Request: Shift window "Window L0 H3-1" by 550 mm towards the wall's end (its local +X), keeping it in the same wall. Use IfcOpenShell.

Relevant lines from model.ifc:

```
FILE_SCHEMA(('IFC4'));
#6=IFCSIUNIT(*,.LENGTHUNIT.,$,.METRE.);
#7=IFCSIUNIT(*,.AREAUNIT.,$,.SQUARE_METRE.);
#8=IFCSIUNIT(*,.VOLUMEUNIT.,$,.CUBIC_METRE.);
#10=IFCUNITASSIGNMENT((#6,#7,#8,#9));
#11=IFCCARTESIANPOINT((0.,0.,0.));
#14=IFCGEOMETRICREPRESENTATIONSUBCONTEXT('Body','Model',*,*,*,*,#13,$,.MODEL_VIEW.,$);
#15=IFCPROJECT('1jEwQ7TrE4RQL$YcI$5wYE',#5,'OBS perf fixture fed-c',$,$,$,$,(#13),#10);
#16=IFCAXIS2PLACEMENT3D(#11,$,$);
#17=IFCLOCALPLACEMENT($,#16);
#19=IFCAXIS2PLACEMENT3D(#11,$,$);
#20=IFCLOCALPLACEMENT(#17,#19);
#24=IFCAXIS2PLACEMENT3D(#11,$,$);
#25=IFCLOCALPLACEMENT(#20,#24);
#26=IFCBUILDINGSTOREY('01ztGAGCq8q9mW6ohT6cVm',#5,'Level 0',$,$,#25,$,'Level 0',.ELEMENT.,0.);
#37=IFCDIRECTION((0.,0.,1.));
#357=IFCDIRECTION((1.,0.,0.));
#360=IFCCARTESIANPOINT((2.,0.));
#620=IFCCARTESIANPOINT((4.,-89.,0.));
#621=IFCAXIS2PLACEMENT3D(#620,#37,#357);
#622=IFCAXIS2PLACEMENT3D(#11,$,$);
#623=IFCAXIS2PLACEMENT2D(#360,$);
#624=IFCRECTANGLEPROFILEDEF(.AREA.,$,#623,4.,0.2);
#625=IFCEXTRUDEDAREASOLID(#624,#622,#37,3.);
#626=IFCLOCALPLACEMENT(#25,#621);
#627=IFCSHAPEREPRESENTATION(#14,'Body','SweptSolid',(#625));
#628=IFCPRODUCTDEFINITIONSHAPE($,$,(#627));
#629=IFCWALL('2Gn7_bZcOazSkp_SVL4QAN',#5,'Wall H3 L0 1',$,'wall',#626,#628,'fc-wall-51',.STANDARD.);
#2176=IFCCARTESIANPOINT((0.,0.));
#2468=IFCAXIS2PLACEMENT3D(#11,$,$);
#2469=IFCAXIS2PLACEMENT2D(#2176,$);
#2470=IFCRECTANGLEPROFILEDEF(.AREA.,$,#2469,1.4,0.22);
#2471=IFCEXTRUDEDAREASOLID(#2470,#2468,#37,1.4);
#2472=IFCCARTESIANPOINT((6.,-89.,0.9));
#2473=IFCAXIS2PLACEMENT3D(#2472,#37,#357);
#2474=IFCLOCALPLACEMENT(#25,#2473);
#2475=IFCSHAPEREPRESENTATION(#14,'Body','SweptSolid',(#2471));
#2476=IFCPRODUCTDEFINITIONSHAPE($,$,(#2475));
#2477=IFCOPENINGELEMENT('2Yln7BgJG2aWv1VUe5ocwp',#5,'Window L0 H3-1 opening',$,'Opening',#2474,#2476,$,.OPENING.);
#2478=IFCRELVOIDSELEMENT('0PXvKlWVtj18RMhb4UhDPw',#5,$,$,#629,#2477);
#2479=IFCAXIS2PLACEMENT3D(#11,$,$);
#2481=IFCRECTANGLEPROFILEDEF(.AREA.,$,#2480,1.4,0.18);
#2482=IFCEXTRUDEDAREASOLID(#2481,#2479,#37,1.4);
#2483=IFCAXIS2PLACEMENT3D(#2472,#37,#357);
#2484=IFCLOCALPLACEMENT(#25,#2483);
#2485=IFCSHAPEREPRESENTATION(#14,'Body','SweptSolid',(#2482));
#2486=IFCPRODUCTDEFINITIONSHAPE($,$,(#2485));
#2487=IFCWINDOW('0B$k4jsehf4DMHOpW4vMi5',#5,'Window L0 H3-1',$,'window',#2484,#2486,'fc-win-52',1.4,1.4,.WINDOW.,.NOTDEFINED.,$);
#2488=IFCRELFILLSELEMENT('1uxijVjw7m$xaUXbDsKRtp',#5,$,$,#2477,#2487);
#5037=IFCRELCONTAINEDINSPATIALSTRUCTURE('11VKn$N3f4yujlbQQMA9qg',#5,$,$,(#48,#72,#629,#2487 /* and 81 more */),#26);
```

```python
import ifcopenshell
import ifcopenshell.api.geometry
import ifcopenshell.util.placement
import ifcopenshell.util.unit

model = ifcopenshell.open("model.ifc")
unit_scale = ifcopenshell.util.unit.calculate_unit_scale(model)

window = model.by_guid("0B$k4jsehf4DMHOpW4vMi5")
opening = window.FillsVoids[0].RelatingOpeningElement
wall = opening.VoidsElements[0].RelatingBuildingElement

wall_matrix = ifcopenshell.util.placement.get_local_placement(wall.ObjectPlacement)
shift = wall_matrix[:3, 0] * 0.55 / unit_scale
before = ifcopenshell.util.placement.get_local_placement(window.ObjectPlacement)[:3, 3].copy()

# The window is not placed relative to its opening, so move both.
for product in (opening, window):
    matrix = ifcopenshell.util.placement.get_local_placement(product.ObjectPlacement)
    matrix[:3, 3] += shift
    ifcopenshell.api.geometry.edit_object_placement(model, product=product, matrix=matrix, is_si=False)

after = ifcopenshell.util.placement.get_local_placement(window.ObjectPlacement)[:3, 3]
print("window moved by", (after - before).round(3) + 0.0)

model.write("model-out.ifc")
```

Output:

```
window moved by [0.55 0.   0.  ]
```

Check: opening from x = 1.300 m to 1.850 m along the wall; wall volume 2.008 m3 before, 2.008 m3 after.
